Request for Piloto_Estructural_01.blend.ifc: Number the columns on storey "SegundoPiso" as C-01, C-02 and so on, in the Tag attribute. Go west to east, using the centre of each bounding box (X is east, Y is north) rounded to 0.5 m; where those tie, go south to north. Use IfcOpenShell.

First a look at what the model holds.

```python
import ifcopenshell
import ifcopenshell.util.element
import ifcopenshell.util.placement

model = ifcopenshell.open("Piloto_Estructural_01.blend.ifc")
print(model.schema)
storey = next(s for s in model.by_type("IfcBuildingStorey") if s.Name == "SegundoPiso")
columns = [e for e in ifcopenshell.util.element.get_decomposition(storey) if e.is_a("IfcColumn")]
for e in sorted(columns, key=lambda e: e.id()):
    origin = ifcopenshell.util.placement.get_local_placement(e.ObjectPlacement)[:3, 3]
    print(e.id(), e.Tag, e.Name, origin.round(2) + 0.0, sep=" | ")
```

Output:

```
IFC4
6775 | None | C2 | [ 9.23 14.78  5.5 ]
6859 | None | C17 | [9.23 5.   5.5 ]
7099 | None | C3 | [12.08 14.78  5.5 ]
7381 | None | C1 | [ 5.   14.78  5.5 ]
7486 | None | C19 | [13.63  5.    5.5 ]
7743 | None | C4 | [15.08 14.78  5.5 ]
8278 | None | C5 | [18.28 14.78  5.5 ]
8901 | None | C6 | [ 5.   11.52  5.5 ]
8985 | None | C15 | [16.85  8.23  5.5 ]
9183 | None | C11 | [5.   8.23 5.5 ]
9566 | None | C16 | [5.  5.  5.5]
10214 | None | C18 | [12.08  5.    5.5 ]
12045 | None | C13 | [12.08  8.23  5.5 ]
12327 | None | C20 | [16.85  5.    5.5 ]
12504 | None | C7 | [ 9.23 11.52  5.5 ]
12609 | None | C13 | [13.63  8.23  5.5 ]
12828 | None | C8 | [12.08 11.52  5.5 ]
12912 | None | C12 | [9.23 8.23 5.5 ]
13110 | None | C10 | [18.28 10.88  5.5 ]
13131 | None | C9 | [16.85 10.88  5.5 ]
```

```python
import ifcopenshell
import ifcopenshell.geom
import ifcopenshell.util.element
import ifcopenshell.util.shape

model = ifcopenshell.open("Piloto_Estructural_01.blend.ifc")
settings = ifcopenshell.geom.settings()
settings.set("use-world-coords", True)


def centre(element):
    shape = ifcopenshell.geom.create_shape(settings, element)
    return ifcopenshell.util.shape.get_bbox_centroid(shape.geometry)


storey = next(s for s in model.by_type("IfcBuildingStorey") if s.Name == "SegundoPiso")
columns = [e for e in ifcopenshell.util.element.get_decomposition(storey) if e.is_a("IfcColumn")]

# Insertion points can sit at a corner or the storey origin, so sort by the geometry (in metres).
centres = {e: centre(e) for e in columns}
columns.sort(key=lambda e: (round(centres[e][0] / 0.5), centres[e][1]))

for i, e in enumerate(columns, start=1):
    number = f"C-{i:02d}"
    e.Tag = number
    print(e.id(), number)

model.write("Piloto_Estructural_01.blend_v2.ifc")
```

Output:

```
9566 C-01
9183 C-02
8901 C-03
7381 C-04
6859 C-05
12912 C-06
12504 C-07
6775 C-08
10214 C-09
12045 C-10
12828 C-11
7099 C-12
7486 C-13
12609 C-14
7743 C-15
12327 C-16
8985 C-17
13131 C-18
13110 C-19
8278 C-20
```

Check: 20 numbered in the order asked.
